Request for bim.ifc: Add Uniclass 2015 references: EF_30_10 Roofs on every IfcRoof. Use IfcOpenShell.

First a look at what the model holds.

```python
import ifcopenshell

model = ifcopenshell.open("bim.ifc")
print(model.schema)
print("classifications:", [c.Name for c in model.by_type("IfcClassification")])
for ifc_class in ("IfcDoor", "IfcRoof", "IfcStair", "IfcWall", "IfcWindow"):
    print(ifc_class, len(model.by_type(ifc_class)))
```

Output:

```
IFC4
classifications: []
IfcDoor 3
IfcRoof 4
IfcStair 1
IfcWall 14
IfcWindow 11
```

```python
import ifcopenshell
import ifcopenshell.api.classification

model = ifcopenshell.open("bim.ifc")

system = ifcopenshell.api.classification.add_classification(model, classification="Uniclass 2015")

codes = {
    "IfcRoof": ("EF_30_10", "Roofs"),
}
for ifc_class, (code, name) in codes.items():
    products = model.by_type(ifc_class)
    ifcopenshell.api.classification.add_reference(
        model, products=products, classification=system, identification=code, name=name
    )
    print(code, len(products))

model.write("bim_v2.ifc")
```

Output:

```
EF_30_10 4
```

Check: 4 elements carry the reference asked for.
